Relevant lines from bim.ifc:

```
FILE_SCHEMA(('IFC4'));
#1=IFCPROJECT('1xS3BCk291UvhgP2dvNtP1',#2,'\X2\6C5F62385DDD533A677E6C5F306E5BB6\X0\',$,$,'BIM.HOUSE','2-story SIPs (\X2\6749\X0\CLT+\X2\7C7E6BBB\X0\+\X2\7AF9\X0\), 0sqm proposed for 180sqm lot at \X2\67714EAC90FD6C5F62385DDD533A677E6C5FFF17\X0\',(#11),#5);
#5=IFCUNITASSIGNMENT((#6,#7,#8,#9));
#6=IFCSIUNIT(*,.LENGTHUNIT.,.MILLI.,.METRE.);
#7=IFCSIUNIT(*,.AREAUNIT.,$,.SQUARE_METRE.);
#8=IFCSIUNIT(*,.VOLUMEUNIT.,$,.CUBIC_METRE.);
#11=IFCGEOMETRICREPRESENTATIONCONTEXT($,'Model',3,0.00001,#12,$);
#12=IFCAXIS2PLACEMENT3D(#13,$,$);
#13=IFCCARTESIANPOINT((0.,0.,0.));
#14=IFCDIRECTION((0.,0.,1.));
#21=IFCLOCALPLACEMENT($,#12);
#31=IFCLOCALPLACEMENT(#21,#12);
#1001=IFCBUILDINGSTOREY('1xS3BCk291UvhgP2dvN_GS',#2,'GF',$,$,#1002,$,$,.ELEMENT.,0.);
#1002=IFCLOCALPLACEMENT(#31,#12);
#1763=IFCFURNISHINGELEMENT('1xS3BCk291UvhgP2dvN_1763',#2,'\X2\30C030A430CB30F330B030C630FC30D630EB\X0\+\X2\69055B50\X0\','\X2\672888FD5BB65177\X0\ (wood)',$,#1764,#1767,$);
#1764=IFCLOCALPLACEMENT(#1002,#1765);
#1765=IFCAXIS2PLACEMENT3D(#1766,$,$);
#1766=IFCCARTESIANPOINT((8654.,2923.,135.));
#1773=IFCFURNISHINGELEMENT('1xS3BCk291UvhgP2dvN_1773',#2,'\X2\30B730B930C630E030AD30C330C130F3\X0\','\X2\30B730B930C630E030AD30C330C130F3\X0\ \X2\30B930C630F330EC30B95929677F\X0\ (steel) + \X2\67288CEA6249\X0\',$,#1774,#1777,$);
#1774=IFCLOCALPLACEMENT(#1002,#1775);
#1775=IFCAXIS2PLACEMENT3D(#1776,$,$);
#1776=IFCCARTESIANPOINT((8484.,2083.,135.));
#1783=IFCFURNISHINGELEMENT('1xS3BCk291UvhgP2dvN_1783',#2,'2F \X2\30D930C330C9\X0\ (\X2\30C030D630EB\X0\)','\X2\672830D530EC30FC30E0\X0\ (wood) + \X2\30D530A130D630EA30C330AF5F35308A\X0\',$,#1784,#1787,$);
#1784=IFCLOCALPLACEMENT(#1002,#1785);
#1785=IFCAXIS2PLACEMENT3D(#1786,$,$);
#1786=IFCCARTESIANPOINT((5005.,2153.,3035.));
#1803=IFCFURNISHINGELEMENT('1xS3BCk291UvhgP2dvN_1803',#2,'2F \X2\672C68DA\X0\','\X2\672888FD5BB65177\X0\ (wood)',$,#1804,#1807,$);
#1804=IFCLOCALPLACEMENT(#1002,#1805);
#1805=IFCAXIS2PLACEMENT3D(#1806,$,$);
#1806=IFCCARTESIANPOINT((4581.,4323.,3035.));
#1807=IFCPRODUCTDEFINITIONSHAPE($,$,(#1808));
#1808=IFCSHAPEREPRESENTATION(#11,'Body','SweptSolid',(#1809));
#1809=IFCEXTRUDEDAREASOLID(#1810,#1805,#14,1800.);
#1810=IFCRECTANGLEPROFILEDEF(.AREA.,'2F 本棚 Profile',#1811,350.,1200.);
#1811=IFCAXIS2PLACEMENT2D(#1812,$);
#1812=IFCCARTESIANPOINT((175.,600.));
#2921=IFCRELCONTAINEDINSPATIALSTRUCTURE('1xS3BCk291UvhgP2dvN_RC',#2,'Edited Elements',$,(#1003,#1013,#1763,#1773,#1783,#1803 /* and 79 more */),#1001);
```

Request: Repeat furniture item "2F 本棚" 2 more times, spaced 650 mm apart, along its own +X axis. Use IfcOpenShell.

```python
import ifcopenshell
import ifcopenshell.api.geometry
import ifcopenshell.api.root
import ifcopenshell.util.element
import ifcopenshell.util.placement
import ifcopenshell.util.unit

model = ifcopenshell.open("bim.ifc")
unit_scale = ifcopenshell.util.unit.calculate_unit_scale(model)


def reuse_history(source, copy):
    """copy_class also copies each property set's owner history, people and application; keep the originals."""
    for rel in copy.IsDefinedBy:
        if rel.is_a("IfcRelDefinesByProperties") and (history := rel.RelatingPropertyDefinition.OwnerHistory):
            rel.RelatingPropertyDefinition.OwnerHistory = source.OwnerHistory
            ifcopenshell.util.element.remove_deep2(model, history)


source = model.by_guid("1xS3BCk291UvhgP2dvN_1803")
base = ifcopenshell.util.placement.get_local_placement(source.ObjectPlacement)
step = base[:3, 0] * 0.65 / unit_scale

for i in range(1, 3):
    copy = ifcopenshell.api.root.copy_class(model, product=source)
    copy.Representation = ifcopenshell.util.element.copy_deep(
        model, source.Representation, exclude=["IfcGeometricRepresentationContext", "IfcRepresentationMap"]
    )
    reuse_history(source, copy)
    matrix = base.copy()
    matrix[:3, 3] += i * step
    print("added at", matrix[:3, 3].round(3) + 0.0)
    ifcopenshell.api.geometry.edit_object_placement(model, product=copy, matrix=matrix, is_si=False)

model.write("bim_v2.ifc")
```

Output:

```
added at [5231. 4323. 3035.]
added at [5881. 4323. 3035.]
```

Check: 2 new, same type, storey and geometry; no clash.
